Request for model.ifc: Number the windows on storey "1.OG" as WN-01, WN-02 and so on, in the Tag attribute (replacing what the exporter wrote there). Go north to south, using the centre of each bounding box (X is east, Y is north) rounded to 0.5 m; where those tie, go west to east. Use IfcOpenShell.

First a look at what the model holds.

```python
import ifcopenshell
import ifcopenshell.util.element
import ifcopenshell.util.placement

model = ifcopenshell.open("model.ifc")
print(model.schema)
storey = next(s for s in model.by_type("IfcBuildingStorey") if s.Name == "1.OG")
windows = [e for e in ifcopenshell.util.element.get_decomposition(storey) if e.is_a("IfcWindow")]
for e in sorted(windows, key=lambda e: e.id()):
    origin = ifcopenshell.util.placement.get_local_placement(e.ObjectPlacement)[:3, 3]
    print(e.id(), e.Tag, e.Name, origin.round(2) + 0.0, sep=" | ")
```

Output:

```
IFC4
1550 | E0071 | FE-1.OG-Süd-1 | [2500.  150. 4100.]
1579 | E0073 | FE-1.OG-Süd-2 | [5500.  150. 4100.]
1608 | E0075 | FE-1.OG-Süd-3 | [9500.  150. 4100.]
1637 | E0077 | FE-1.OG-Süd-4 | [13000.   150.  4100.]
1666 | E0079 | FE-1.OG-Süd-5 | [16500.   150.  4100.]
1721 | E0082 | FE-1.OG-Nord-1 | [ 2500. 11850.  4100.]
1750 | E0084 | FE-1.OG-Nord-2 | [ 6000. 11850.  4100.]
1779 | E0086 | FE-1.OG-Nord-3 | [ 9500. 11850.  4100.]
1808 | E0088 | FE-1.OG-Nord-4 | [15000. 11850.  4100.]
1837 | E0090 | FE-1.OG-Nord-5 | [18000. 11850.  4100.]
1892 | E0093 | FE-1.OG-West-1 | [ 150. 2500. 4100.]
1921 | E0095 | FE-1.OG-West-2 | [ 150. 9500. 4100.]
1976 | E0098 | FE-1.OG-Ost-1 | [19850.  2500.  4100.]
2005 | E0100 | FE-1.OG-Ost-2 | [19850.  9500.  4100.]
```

```python
import ifcopenshell
import ifcopenshell.geom
import ifcopenshell.util.element
import ifcopenshell.util.shape

model = ifcopenshell.open("model.ifc")
settings = ifcopenshell.geom.settings()
settings.set("use-world-coords", True)


def centre(element):
    shape = ifcopenshell.geom.create_shape(settings, element)
    return ifcopenshell.util.shape.get_bbox_centroid(shape.geometry)


storey = next(s for s in model.by_type("IfcBuildingStorey") if s.Name == "1.OG")
windows = [e for e in ifcopenshell.util.element.get_decomposition(storey) if e.is_a("IfcWindow")]

# Insertion points can sit at a corner or the storey origin, so sort by the geometry (in metres).
centres = {e: centre(e) for e in windows}
windows.sort(key=lambda e: (-round(centres[e][1] / 0.5), centres[e][0]))

for i, e in enumerate(windows, start=1):
    number = f"WN-{i:02d}"
    e.Tag = number
    print(e.id(), number)

model.write("model-out.ifc")
```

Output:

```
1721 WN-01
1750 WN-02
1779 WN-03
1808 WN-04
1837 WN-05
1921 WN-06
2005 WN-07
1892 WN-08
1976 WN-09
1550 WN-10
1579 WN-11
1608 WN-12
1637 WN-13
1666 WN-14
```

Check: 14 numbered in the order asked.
